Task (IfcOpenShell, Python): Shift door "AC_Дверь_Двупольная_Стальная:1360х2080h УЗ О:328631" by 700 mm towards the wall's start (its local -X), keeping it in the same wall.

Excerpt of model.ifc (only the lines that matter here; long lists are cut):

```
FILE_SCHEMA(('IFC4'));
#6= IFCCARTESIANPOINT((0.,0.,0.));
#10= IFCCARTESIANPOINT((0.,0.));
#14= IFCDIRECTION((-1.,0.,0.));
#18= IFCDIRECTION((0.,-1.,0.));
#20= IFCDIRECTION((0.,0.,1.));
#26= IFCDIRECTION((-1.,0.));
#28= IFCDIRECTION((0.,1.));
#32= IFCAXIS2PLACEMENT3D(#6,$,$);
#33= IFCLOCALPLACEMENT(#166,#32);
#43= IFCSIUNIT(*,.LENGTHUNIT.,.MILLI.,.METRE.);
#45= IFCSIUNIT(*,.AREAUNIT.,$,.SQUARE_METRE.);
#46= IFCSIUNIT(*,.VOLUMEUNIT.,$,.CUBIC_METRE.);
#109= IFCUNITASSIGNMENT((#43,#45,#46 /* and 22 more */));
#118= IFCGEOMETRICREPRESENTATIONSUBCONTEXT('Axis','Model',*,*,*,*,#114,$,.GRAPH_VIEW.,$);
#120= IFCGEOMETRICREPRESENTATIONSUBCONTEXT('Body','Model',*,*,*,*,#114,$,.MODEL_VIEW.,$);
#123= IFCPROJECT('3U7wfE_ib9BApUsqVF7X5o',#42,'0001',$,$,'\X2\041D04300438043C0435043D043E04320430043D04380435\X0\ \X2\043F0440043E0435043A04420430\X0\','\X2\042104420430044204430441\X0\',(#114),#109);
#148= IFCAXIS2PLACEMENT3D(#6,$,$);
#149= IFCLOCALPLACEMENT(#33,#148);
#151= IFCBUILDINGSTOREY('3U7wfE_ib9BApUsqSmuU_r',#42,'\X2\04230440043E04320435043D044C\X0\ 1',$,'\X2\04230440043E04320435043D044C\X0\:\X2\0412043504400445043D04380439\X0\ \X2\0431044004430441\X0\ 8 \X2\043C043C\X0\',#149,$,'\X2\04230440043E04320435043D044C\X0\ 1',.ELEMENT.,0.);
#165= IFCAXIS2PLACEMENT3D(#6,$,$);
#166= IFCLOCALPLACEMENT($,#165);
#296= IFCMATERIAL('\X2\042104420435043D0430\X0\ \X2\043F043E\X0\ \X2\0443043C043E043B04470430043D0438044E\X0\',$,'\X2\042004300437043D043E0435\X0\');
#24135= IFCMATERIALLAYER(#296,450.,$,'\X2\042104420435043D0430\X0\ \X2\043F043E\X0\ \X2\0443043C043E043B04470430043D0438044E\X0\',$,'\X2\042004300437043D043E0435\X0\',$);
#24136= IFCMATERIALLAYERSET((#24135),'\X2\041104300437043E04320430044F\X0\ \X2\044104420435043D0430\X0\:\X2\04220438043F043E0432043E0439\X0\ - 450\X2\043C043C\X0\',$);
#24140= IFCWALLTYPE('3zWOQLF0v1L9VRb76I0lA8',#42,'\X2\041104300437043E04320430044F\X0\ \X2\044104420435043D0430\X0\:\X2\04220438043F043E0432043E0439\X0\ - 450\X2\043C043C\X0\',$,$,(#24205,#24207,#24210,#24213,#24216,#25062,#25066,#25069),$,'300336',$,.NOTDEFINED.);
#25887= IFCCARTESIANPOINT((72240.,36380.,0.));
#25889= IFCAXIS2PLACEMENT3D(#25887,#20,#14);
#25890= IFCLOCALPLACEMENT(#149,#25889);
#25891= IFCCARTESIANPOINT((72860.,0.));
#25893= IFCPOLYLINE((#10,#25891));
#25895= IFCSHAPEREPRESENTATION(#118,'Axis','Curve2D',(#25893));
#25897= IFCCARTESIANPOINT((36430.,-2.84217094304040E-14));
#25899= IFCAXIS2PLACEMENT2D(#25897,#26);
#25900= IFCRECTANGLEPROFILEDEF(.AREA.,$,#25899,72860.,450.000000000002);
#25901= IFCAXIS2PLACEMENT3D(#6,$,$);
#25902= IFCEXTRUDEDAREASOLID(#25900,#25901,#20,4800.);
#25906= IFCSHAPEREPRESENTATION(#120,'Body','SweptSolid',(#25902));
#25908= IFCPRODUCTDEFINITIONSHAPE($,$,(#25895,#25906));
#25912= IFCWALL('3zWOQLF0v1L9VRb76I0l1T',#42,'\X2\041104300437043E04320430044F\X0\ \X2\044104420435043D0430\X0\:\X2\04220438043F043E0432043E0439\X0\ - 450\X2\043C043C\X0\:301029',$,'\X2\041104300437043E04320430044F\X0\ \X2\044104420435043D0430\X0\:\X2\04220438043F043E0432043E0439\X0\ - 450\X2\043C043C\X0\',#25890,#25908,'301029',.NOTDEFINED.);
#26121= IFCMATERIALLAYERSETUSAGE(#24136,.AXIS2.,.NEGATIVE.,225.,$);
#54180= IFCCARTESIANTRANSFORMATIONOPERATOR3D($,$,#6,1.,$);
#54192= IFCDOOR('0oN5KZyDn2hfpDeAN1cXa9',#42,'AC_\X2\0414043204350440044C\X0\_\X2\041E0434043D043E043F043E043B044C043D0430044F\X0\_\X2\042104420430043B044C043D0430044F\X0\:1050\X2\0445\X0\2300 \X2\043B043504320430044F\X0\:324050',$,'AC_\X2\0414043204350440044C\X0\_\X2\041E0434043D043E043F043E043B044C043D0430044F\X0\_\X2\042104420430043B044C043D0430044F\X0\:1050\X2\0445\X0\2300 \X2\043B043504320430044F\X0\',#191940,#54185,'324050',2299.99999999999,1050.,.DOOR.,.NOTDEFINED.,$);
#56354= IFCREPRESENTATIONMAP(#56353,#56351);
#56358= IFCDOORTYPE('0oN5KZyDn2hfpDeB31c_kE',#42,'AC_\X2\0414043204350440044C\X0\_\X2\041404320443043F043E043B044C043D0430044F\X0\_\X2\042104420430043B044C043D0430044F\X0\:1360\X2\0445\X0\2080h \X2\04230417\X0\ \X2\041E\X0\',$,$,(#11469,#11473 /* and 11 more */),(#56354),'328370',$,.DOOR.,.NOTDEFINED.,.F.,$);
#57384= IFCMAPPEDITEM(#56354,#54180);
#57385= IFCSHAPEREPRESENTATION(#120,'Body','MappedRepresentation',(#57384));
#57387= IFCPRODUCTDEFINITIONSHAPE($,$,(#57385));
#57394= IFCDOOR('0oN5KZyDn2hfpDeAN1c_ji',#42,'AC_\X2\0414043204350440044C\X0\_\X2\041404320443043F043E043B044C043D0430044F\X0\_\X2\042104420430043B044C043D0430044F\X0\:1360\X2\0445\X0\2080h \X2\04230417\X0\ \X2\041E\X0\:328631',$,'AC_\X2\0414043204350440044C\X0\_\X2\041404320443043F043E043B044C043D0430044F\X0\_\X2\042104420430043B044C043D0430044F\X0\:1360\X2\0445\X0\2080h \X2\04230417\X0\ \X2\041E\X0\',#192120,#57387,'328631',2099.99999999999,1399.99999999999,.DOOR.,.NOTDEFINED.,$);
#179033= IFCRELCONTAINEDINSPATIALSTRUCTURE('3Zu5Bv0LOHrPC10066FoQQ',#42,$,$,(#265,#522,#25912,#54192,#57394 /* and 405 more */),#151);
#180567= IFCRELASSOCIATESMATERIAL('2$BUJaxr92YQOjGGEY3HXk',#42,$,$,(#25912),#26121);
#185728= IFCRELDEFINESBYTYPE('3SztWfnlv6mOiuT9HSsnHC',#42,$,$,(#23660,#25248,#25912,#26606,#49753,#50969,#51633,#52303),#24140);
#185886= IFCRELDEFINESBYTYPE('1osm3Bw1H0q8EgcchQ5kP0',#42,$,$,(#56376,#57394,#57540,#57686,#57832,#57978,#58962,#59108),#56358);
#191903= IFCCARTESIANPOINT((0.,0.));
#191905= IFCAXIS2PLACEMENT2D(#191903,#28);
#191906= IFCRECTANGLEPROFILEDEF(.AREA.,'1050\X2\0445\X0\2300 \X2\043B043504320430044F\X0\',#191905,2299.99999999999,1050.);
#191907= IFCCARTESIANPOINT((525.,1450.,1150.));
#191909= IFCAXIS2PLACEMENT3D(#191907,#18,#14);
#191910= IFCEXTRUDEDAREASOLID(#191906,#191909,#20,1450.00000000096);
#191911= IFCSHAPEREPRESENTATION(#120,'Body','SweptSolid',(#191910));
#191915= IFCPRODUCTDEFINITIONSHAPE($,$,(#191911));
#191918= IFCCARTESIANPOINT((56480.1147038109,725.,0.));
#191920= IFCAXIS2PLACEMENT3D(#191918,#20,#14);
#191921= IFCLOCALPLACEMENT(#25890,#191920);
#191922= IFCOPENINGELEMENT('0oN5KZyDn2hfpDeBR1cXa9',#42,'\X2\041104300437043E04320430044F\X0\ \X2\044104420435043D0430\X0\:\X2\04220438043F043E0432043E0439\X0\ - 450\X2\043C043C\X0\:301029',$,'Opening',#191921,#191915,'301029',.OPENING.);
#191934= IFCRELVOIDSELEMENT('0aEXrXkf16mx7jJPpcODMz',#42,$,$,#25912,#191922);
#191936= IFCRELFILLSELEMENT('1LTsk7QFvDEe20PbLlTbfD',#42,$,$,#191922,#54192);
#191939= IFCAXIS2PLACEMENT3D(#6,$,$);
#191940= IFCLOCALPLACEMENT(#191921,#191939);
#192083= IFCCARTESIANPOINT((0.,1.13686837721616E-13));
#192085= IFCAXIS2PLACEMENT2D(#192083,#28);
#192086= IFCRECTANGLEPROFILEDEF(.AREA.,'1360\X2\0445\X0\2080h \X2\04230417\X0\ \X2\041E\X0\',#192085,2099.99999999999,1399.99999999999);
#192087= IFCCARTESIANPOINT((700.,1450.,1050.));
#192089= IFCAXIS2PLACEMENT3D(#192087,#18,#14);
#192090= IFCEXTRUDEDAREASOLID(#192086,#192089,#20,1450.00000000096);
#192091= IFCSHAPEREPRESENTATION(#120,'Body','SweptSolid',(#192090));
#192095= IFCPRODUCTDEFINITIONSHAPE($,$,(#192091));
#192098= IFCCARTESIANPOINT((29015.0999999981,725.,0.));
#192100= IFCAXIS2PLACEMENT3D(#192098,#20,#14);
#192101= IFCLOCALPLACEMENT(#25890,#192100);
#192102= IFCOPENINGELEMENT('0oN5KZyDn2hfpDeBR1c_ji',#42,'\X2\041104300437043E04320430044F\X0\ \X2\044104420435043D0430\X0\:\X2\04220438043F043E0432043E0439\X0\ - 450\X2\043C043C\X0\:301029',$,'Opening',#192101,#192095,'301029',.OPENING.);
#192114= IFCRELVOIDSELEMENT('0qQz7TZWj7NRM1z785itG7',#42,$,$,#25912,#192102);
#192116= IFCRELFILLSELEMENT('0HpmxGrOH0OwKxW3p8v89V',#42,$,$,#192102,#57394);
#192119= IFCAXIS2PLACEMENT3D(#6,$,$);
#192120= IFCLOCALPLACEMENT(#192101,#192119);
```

```python
import ifcopenshell
import ifcopenshell.api.geometry
import ifcopenshell.util.placement
import ifcopenshell.util.unit

model = ifcopenshell.open("model.ifc")
unit_scale = ifcopenshell.util.unit.calculate_unit_scale(model)

door = model.by_guid("0oN5KZyDn2hfpDeAN1c_ji")
opening = door.FillsVoids[0].RelatingOpeningElement
wall = opening.VoidsElements[0].RelatingBuildingElement

wall_matrix = ifcopenshell.util.placement.get_local_placement(wall.ObjectPlacement)
shift = wall_matrix[:3, 0] * -0.7 / unit_scale
before = ifcopenshell.util.placement.get_local_placement(door.ObjectPlacement)[:3, 3].copy()

# The door is placed relative to its opening, so it follows when the opening moves.
matrix = ifcopenshell.util.placement.get_local_placement(opening.ObjectPlacement)
matrix[:3, 3] += shift
ifcopenshell.api.geometry.edit_object_placement(
    model, product=opening, matrix=matrix, is_si=False, should_transform_children=True
)

after = ifcopenshell.util.placement.get_local_placement(door.ObjectPlacement)[:3, 3]
print("door moved by", (after - before).round(3) + 0.0)

model.write("model_v2.ifc")
```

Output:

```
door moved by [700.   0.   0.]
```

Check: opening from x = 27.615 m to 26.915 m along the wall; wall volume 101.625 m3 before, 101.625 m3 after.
